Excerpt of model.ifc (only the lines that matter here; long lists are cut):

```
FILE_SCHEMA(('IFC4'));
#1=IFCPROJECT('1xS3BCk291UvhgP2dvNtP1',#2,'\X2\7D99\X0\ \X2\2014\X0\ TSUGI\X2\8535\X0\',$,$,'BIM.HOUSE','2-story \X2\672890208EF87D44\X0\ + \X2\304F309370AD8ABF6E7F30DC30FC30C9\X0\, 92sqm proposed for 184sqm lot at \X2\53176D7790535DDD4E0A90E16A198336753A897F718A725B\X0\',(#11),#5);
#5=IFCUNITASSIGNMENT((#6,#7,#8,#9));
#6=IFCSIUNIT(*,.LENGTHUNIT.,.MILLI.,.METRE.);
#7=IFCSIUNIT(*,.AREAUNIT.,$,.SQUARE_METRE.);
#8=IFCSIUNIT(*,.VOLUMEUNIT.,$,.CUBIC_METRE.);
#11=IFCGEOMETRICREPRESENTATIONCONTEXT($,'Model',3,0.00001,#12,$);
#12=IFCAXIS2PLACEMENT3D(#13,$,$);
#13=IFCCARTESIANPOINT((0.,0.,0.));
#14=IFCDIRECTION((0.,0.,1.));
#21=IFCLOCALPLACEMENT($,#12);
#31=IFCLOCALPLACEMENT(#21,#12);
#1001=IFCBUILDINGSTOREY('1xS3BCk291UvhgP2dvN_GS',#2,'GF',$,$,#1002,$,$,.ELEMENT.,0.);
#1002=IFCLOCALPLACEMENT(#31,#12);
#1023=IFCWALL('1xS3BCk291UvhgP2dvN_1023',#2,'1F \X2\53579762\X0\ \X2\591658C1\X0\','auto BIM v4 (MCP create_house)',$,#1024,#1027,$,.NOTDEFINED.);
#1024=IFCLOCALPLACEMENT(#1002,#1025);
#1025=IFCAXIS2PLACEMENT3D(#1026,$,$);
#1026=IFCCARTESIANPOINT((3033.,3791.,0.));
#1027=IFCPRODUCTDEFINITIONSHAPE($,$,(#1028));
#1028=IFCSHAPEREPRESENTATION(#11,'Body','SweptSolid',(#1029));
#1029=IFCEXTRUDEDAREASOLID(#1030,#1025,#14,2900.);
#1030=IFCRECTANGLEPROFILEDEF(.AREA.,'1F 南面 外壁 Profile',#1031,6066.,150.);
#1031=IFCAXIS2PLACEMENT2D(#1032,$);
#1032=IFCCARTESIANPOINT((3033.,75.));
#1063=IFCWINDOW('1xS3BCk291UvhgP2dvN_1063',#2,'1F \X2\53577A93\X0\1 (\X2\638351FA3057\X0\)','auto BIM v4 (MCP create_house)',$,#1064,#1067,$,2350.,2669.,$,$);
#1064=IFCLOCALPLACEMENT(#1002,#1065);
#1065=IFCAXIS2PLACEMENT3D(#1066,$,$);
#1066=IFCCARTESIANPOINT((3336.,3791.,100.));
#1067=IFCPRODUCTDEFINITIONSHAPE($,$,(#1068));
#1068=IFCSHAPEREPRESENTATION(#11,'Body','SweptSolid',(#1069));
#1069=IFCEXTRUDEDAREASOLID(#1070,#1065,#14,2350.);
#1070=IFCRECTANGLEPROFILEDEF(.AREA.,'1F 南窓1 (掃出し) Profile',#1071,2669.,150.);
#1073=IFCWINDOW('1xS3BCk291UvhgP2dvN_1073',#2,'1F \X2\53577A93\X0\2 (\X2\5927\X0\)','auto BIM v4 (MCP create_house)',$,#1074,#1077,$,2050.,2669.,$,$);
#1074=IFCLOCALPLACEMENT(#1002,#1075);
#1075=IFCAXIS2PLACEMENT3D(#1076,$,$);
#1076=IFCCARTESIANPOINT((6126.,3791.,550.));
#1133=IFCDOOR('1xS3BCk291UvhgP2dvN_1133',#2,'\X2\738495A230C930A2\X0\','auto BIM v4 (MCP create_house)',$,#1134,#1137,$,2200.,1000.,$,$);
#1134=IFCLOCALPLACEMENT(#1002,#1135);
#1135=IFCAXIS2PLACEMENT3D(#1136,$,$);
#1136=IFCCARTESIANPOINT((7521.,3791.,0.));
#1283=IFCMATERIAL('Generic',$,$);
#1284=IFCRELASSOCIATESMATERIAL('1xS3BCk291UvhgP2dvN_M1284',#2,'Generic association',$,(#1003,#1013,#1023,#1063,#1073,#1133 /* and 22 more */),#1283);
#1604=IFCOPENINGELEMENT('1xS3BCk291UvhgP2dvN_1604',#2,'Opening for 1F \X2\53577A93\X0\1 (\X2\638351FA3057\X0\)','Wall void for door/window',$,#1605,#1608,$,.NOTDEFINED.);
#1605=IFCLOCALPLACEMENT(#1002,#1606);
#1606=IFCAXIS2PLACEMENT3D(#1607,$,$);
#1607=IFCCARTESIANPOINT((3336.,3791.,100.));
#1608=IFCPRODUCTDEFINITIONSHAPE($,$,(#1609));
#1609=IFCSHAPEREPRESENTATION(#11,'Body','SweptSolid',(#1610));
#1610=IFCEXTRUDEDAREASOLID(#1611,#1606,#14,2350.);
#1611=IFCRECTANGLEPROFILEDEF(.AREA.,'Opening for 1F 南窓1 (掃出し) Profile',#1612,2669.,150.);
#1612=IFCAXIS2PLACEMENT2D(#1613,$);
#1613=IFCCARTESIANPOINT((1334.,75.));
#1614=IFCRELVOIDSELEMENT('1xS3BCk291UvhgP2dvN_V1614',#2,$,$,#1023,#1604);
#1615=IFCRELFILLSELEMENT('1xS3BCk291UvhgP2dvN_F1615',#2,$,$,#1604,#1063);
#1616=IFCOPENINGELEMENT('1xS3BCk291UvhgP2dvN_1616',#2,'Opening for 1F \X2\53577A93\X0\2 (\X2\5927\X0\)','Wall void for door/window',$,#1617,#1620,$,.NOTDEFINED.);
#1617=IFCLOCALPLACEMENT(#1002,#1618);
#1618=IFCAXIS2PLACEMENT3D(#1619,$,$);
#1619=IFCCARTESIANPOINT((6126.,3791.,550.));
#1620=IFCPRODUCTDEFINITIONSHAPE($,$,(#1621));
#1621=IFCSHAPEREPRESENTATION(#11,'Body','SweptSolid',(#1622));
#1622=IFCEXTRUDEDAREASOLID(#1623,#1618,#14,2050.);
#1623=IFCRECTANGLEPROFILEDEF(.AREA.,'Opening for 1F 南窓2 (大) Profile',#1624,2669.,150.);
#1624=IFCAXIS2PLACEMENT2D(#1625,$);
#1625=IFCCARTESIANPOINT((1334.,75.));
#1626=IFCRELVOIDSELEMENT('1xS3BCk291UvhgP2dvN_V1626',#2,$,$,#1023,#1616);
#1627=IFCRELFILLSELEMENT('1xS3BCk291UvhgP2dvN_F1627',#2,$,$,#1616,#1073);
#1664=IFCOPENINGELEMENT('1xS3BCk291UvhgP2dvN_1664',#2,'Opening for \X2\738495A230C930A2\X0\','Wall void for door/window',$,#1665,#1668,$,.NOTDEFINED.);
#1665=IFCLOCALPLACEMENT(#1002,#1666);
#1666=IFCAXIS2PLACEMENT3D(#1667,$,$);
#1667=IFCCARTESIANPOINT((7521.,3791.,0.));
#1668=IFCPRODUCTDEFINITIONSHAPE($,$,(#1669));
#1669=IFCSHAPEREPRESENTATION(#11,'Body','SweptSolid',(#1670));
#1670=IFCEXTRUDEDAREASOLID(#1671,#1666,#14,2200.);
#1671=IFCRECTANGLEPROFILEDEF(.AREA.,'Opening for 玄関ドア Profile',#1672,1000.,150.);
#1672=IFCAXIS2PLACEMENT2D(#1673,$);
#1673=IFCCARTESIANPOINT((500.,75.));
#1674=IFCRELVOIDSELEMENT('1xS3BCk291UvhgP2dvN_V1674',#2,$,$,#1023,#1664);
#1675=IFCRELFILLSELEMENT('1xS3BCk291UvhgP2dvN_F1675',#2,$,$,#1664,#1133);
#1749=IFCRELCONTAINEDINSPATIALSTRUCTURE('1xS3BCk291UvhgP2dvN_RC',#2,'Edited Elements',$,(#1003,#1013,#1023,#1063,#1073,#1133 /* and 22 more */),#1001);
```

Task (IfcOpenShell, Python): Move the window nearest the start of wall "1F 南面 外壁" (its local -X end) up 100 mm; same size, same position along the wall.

```python
import numpy as np
import ifcopenshell
import ifcopenshell.api.geometry
import ifcopenshell.util.placement
import ifcopenshell.util.unit

model = ifcopenshell.open("model.ifc")
unit_scale = ifcopenshell.util.unit.calculate_unit_scale(model)

window = model.by_guid("1xS3BCk291UvhgP2dvN_1063")
opening = window.FillsVoids[0].RelatingOpeningElement
dz = 100.0

shift = np.array([0.0, 0.0, dz])
# The window is not placed relative to its opening, so move both.
for product in (opening, window):
    matrix = ifcopenshell.util.placement.get_local_placement(product.ObjectPlacement)
    matrix[:3, 3] += shift
    ifcopenshell.api.geometry.edit_object_placement(model, product=product, matrix=matrix, is_si=False)

print(f"moved by {dz * unit_scale:+.3f} m")

model.write("model_v2.ifc")
```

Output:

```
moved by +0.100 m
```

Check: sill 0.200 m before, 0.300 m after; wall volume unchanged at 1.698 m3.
